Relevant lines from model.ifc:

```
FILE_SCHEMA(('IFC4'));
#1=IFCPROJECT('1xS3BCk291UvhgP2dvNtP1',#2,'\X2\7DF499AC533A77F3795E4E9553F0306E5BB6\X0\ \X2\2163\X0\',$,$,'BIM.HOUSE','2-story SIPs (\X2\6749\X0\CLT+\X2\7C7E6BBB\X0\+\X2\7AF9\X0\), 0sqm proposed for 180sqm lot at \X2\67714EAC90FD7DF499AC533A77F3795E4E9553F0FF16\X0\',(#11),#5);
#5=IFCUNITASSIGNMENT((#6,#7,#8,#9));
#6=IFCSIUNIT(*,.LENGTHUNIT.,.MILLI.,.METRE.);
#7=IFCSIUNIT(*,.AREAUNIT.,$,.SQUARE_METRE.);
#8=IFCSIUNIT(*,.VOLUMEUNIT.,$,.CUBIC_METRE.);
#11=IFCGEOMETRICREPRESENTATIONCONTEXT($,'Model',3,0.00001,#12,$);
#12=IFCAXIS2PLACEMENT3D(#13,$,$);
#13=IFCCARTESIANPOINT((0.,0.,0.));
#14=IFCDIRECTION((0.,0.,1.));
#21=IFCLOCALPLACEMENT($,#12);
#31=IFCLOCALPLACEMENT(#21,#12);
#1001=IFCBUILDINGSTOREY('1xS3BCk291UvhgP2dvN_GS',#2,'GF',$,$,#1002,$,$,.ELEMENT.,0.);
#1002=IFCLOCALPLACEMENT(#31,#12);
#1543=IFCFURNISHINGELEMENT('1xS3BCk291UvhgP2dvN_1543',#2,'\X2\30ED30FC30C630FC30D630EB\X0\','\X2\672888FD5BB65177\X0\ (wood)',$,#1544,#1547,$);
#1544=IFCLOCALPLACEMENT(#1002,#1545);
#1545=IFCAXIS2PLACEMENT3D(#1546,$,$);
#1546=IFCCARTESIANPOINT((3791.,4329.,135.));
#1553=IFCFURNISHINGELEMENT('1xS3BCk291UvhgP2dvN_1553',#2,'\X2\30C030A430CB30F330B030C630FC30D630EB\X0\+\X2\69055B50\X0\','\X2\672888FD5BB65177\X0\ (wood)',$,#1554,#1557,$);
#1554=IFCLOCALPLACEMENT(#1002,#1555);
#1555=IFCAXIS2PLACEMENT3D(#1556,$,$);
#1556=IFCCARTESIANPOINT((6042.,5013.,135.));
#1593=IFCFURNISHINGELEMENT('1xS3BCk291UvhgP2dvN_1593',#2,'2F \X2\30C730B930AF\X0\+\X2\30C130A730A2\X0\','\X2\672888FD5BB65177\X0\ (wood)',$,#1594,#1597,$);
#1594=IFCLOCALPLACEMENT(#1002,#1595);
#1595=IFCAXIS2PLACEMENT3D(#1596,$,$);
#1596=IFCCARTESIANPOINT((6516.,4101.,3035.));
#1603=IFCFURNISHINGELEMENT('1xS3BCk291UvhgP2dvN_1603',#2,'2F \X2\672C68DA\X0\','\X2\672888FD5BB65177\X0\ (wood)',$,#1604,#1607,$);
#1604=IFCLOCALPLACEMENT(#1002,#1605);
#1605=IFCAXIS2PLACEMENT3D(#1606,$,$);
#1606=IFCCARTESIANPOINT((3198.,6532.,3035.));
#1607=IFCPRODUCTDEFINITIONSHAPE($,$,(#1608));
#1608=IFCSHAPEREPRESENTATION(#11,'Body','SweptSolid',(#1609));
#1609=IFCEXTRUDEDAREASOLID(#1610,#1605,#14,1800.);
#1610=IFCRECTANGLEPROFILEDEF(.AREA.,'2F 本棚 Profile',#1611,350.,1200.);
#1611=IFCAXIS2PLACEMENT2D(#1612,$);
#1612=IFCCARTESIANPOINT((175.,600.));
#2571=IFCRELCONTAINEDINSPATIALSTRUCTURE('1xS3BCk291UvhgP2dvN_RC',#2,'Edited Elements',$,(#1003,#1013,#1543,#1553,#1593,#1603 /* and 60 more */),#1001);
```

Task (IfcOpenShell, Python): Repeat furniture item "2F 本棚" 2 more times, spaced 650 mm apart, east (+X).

```python
import numpy as np
import ifcopenshell
import ifcopenshell.api.geometry
import ifcopenshell.api.root
import ifcopenshell.util.element
import ifcopenshell.util.placement

model = ifcopenshell.open("model.ifc")


def reuse_history(source, copy):
    """copy_class also copies each property set's owner history, people and application; keep the originals."""
    for rel in copy.IsDefinedBy:
        if rel.is_a("IfcRelDefinesByProperties") and (history := rel.RelatingPropertyDefinition.OwnerHistory):
            rel.RelatingPropertyDefinition.OwnerHistory = source.OwnerHistory
            ifcopenshell.util.element.remove_deep2(model, history)


source = model.by_guid("1xS3BCk291UvhgP2dvN_1603")
base = ifcopenshell.util.placement.get_local_placement(source.ObjectPlacement)
step = np.array([1.0, 0.0, 0.0]) * 650.0

for i in range(1, 3):
    copy = ifcopenshell.api.root.copy_class(model, product=source)
    copy.Representation = ifcopenshell.util.element.copy_deep(
        model, source.Representation, exclude=["IfcGeometricRepresentationContext", "IfcRepresentationMap"]
    )
    reuse_history(source, copy)
    matrix = base.copy()
    matrix[:3, 3] += i * step
    print("added at", matrix[:3, 3].round(3) + 0.0)
    ifcopenshell.api.geometry.edit_object_placement(model, product=copy, matrix=matrix, is_si=False)

model.write("model_v2.ifc")
```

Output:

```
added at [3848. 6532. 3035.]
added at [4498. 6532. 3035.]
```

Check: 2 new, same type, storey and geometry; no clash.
